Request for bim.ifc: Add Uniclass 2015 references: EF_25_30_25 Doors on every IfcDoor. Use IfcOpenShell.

First a look at what the model holds.

```python
import ifcopenshell

model = ifcopenshell.open("bim.ifc")
print(model.schema)
print("classifications:", [c.Name for c in model.by_type("IfcClassification")])
for ifc_class in ("IfcDoor", "IfcRoof", "IfcStair", "IfcWall", "IfcWindow"):
    print(ifc_class, len(model.by_type(ifc_class)))
```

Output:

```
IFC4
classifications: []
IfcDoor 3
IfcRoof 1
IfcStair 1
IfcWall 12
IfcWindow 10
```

```python
import ifcopenshell
import ifcopenshell.api.classification

model = ifcopenshell.open("bim.ifc")

system = ifcopenshell.api.classification.add_classification(model, classification="Uniclass 2015")

codes = {
    "IfcDoor": ("EF_25_30_25", "Doors"),
}
for ifc_class, (code, name) in codes.items():
    products = model.by_type(ifc_class)
    ifcopenshell.api.classification.add_reference(
        model, products=products, classification=system, identification=code, name=name
    )
    print(code, len(products))

model.write("bim_rev.ifc")
```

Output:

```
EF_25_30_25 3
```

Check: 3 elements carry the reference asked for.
